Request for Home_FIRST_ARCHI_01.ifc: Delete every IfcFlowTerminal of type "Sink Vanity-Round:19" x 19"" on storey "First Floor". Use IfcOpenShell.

First a look at what the model holds.

```python
import ifcopenshell
import ifcopenshell.util.element

model = ifcopenshell.open("Home_FIRST_ARCHI_01.ifc")
print(model.schema)
storey = next(s for s in model.by_type("IfcBuildingStorey") if s.Name == "First Floor")
terminals = [e for e in ifcopenshell.util.element.get_decomposition(storey) if e.is_a("IfcFlowTerminal")]
seen = {}
for e in terminals:
    element_type = ifcopenshell.util.element.get_type(e)
    name = element_type.Name if element_type not in (None, e) else None
    seen[name] = seen.get(name, 0) + 1
for name, count in sorted(seen.items(), key=str):
    print(count, "x", name)
```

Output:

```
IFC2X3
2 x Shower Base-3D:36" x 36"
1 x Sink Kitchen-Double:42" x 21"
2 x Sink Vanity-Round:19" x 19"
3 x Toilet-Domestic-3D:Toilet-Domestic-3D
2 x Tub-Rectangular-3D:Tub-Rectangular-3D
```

```python
import ifcopenshell
import ifcopenshell.api.root
import ifcopenshell.util.element

model = ifcopenshell.open("Home_FIRST_ARCHI_01.ifc")

storey = next(s for s in model.by_type("IfcBuildingStorey") if s.Name == "First Floor")
terminals = [e for e in ifcopenshell.util.element.get_decomposition(storey) if e.is_a("IfcFlowTerminal")]
targets = [e for e in terminals if (t := ifcopenshell.util.element.get_type(e)) not in (None, e) and t.Name == 'Sink Vanity-Round:19" x 19"']

for e in targets:
    ifcopenshell.api.root.remove_product(model, product=e)
print(len(targets), "removed")

model.write("Home_FIRST_ARCHI_01-out.ifc")
```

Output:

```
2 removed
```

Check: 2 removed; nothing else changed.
